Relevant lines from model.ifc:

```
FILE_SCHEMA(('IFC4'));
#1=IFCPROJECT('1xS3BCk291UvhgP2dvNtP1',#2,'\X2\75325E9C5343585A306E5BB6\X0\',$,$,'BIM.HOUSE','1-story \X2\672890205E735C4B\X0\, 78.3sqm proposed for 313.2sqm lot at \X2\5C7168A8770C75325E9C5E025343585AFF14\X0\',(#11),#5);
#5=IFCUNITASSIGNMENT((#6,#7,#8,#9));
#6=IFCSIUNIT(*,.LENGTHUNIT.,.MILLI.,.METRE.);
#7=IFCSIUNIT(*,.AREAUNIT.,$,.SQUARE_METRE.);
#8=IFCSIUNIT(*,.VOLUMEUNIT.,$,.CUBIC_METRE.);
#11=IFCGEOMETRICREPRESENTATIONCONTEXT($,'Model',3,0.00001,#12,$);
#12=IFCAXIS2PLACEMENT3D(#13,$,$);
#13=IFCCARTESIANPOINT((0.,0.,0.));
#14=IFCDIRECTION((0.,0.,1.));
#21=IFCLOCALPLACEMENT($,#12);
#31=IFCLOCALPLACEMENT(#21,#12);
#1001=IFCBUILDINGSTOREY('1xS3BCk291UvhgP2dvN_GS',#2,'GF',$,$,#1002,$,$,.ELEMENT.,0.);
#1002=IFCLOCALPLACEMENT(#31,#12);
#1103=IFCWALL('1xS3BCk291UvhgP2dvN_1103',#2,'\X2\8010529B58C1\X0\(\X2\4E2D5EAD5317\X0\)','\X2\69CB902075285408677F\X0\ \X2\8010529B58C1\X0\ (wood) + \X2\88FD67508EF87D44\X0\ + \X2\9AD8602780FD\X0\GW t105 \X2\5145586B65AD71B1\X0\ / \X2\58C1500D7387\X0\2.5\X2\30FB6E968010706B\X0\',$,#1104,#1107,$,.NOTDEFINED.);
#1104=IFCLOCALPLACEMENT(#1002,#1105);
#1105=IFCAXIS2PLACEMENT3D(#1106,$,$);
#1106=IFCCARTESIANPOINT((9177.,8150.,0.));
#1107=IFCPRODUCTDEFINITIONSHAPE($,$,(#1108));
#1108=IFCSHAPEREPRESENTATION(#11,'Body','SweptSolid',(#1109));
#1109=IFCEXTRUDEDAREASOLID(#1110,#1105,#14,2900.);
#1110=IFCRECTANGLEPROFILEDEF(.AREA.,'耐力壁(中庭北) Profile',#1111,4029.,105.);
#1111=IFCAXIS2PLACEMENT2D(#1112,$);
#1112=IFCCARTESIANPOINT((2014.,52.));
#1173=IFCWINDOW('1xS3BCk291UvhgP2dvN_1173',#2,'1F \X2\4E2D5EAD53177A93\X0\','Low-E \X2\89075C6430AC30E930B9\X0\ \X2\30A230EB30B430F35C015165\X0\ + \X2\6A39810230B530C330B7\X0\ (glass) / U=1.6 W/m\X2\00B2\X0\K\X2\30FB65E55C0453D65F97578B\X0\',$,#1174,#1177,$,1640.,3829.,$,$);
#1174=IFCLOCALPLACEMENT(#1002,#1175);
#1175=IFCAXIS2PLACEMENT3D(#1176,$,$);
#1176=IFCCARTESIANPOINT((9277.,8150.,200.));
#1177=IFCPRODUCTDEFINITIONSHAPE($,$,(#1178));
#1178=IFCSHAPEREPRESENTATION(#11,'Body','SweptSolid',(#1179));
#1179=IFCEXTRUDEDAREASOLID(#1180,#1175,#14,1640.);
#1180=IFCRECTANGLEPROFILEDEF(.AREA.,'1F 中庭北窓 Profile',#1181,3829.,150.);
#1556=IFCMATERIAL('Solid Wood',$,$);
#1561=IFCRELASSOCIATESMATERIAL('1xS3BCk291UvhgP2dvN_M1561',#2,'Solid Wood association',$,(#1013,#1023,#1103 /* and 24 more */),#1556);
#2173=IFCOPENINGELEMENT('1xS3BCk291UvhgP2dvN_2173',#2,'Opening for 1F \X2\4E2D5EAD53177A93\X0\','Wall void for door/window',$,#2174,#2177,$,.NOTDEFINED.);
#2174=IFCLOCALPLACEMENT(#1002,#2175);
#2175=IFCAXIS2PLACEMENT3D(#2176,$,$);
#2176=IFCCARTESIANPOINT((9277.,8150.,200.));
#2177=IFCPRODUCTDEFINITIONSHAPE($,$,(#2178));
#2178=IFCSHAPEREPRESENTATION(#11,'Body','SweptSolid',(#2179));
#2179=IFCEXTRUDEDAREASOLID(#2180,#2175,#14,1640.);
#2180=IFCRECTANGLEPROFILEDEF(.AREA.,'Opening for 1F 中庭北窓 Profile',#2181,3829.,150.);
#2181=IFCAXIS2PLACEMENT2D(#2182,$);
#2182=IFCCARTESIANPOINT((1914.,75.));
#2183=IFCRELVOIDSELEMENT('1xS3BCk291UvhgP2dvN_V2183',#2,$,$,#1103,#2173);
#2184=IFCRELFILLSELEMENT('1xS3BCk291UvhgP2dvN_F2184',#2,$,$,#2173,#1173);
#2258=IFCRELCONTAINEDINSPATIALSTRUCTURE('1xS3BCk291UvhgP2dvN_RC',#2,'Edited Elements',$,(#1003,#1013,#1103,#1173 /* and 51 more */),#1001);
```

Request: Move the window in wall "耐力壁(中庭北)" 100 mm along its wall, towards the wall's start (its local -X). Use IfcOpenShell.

```python
import ifcopenshell
import ifcopenshell.api.geometry
import ifcopenshell.util.placement

model = ifcopenshell.open("model.ifc")

window = model.by_id(1173)
opening = window.FillsVoids[0].RelatingOpeningElement
wall = opening.VoidsElements[0].RelatingBuildingElement

wall_matrix = ifcopenshell.util.placement.get_local_placement(wall.ObjectPlacement)
shift = wall_matrix[:3, 0] * -100.0
before = ifcopenshell.util.placement.get_local_placement(window.ObjectPlacement)[:3, 3].copy()

# The window is not placed relative to its opening, so move both.
for product in (opening, window):
    matrix = ifcopenshell.util.placement.get_local_placement(product.ObjectPlacement)
    matrix[:3, 3] += shift
    ifcopenshell.api.geometry.edit_object_placement(model, product=product, matrix=matrix, is_si=False)

after = ifcopenshell.util.placement.get_local_placement(window.ObjectPlacement)[:3, 3]
print("window moved by", (after - before).round(3) + 0.0)

model.write("model_edited.ifc")
```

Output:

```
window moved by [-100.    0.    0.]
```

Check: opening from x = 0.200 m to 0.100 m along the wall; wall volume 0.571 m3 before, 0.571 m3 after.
